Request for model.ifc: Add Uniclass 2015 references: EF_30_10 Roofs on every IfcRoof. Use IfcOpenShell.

First a look at what the model holds.

```python
import ifcopenshell

model = ifcopenshell.open("model.ifc")
print(model.schema)
print("classifications:", [c.Name for c in model.by_type("IfcClassification")])
for ifc_class in ("IfcDoor", "IfcRoof", "IfcStair", "IfcWall", "IfcWindow"):
    print(ifc_class, len(model.by_type(ifc_class)))
```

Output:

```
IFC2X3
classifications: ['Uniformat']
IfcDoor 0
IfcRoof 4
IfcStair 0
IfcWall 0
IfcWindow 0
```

```python
import ifcopenshell
import ifcopenshell.api.classification

model = ifcopenshell.open("model.ifc")

# IFC2X3 requires Source and Edition and has no link from the project to the system.
system = model.create_entity("IfcClassification", Source="NBS", Edition="2015", Name="Uniclass 2015")

codes = {
    "IfcRoof": ("EF_30_10", "Roofs"),
}
for ifc_class, (code, name) in codes.items():
    products = model.by_type(ifc_class)
    ifcopenshell.api.classification.add_reference(
        model, products=products, classification=system, identification=code, name=name
    )
    print(code, len(products))

model.write("model_edited.ifc")
```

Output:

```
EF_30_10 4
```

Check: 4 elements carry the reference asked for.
